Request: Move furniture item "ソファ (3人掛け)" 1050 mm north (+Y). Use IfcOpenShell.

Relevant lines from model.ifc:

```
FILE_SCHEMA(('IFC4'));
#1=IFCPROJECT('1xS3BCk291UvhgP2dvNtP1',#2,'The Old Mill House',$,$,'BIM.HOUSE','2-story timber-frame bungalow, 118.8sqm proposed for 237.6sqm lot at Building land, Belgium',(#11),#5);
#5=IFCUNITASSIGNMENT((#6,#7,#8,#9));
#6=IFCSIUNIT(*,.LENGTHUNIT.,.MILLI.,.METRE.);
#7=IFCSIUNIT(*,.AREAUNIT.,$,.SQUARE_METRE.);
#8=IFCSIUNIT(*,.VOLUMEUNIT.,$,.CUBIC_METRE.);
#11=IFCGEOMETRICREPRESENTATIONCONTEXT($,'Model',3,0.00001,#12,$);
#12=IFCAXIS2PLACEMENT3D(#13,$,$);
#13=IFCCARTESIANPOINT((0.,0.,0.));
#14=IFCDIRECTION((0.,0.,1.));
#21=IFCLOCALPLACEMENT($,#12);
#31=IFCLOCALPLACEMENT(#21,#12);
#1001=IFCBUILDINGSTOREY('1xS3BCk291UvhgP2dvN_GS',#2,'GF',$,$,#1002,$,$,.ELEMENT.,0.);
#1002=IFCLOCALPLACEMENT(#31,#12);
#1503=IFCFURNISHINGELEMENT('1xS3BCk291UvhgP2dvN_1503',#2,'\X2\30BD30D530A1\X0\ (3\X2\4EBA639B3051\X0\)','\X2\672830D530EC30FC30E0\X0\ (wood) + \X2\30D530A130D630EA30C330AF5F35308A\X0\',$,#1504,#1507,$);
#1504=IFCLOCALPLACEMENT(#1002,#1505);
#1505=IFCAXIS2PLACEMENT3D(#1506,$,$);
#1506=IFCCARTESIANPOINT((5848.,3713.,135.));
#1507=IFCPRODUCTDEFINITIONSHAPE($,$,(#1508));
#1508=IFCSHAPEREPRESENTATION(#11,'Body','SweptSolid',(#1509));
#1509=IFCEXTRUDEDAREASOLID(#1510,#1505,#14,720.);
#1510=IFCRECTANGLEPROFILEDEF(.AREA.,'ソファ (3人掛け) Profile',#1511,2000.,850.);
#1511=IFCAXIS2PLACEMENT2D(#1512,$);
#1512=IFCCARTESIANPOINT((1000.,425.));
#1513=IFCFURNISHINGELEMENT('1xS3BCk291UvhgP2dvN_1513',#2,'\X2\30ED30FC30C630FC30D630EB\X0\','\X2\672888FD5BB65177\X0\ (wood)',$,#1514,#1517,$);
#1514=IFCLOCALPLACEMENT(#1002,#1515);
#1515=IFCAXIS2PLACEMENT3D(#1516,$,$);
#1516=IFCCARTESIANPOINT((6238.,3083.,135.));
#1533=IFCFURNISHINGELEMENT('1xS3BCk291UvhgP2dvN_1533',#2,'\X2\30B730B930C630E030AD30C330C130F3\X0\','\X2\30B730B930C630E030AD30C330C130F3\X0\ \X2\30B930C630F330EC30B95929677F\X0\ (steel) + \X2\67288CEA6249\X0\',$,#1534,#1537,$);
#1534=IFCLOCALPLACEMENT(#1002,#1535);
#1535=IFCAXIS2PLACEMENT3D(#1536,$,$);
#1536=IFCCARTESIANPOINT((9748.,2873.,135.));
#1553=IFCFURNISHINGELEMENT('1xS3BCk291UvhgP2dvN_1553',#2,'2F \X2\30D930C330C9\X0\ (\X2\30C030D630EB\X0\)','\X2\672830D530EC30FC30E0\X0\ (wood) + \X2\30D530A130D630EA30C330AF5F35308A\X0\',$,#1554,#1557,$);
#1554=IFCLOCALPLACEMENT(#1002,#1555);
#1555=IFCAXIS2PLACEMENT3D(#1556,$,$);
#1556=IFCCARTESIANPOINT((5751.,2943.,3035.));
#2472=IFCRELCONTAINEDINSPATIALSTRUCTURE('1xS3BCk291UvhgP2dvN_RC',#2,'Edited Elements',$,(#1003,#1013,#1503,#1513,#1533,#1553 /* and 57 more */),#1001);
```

```python
import ifcopenshell
import ifcopenshell.api.geometry
import ifcopenshell.util.placement
import ifcopenshell.util.unit

model = ifcopenshell.open("model.ifc")
unit_scale = ifcopenshell.util.unit.calculate_unit_scale(model)

item = model.by_id(1503)
matrix = ifcopenshell.util.placement.get_local_placement(item.ObjectPlacement)
matrix[1, 3] += 1.05 / unit_scale
ifcopenshell.api.geometry.edit_object_placement(model, product=item, matrix=matrix, is_si=False)

print(ifcopenshell.util.placement.get_local_placement(item.ObjectPlacement).round(3) + 0.0)

model.write("model_v2.ifc")
```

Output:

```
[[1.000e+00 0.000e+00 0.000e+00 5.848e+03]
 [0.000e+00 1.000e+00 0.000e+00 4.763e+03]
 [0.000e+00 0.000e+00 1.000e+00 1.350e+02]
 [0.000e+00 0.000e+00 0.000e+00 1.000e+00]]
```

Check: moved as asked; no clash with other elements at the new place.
